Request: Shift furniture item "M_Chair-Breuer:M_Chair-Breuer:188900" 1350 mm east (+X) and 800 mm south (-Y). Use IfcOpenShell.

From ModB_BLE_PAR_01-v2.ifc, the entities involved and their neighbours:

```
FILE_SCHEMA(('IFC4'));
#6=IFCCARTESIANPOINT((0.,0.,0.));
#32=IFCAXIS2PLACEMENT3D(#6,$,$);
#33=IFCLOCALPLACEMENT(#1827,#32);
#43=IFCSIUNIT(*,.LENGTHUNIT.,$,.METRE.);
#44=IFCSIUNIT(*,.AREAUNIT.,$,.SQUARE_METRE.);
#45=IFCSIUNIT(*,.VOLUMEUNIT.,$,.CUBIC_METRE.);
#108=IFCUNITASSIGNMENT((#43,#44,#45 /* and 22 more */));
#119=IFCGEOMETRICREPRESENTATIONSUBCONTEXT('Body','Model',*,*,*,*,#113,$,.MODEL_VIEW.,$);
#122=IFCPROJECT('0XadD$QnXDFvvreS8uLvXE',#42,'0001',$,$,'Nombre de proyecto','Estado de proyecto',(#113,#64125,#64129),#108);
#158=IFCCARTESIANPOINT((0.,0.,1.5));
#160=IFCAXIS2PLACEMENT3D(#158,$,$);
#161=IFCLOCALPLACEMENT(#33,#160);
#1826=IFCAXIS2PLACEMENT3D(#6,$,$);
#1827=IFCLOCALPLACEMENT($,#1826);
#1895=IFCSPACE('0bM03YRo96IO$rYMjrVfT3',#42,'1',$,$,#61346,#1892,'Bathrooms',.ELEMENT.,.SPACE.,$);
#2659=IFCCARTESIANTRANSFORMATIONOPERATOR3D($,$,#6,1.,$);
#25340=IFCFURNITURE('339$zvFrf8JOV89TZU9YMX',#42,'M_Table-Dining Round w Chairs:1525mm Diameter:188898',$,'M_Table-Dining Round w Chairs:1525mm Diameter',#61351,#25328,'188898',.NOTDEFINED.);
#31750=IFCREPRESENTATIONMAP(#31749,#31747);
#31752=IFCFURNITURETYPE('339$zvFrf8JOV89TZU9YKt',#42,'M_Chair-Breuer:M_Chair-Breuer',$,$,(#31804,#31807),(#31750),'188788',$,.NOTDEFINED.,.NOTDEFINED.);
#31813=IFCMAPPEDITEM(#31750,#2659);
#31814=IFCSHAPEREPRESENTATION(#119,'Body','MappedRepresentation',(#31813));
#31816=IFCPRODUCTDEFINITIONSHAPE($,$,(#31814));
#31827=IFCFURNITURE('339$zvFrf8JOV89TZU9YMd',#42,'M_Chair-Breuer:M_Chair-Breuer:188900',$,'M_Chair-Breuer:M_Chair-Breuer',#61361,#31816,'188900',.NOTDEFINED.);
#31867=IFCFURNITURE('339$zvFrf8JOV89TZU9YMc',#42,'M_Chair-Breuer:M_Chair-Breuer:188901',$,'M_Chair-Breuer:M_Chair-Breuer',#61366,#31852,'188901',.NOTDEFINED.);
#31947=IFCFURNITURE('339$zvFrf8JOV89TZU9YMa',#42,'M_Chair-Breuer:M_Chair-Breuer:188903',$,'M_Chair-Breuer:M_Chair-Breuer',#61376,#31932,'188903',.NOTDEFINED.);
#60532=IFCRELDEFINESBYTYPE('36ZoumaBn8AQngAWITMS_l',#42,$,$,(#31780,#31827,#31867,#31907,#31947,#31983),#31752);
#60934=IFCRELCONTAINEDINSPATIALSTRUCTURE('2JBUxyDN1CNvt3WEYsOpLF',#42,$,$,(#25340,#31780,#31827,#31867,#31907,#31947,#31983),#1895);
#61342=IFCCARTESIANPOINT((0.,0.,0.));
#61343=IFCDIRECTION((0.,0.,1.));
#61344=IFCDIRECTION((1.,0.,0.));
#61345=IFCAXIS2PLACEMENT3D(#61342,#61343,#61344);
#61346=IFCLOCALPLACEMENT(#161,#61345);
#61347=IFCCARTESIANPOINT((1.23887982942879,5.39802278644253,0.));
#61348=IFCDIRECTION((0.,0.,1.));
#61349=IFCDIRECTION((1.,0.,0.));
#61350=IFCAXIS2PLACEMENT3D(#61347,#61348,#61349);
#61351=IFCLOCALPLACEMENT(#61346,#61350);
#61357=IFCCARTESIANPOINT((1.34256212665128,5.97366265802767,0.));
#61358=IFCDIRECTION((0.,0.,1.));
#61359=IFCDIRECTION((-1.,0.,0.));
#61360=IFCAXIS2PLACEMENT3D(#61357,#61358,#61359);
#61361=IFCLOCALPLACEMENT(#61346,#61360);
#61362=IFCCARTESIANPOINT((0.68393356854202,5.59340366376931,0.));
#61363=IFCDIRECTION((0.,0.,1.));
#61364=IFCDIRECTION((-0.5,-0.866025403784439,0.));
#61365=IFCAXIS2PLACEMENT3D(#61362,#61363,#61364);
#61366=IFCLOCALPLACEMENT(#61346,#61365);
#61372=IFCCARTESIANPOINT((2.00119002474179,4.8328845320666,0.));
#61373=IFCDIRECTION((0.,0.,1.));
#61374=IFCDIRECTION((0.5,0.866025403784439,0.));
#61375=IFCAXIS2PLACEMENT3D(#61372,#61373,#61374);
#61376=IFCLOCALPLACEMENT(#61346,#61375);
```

```python
import ifcopenshell
import ifcopenshell.api.geometry
import ifcopenshell.util.placement
import ifcopenshell.util.unit

model = ifcopenshell.open("ModB_BLE_PAR_01-v2.ifc")
unit_scale = ifcopenshell.util.unit.calculate_unit_scale(model)

item = model.by_guid("339$zvFrf8JOV89TZU9YMd")
matrix = ifcopenshell.util.placement.get_local_placement(item.ObjectPlacement)
matrix[0, 3] += 1.35 / unit_scale
matrix[1, 3] -= 0.8 / unit_scale
ifcopenshell.api.geometry.edit_object_placement(model, product=item, matrix=matrix, is_si=False)

print(ifcopenshell.util.placement.get_local_placement(item.ObjectPlacement).round(3) + 0.0)

model.write("ModB_BLE_PAR_01-v2_edited.ifc")
```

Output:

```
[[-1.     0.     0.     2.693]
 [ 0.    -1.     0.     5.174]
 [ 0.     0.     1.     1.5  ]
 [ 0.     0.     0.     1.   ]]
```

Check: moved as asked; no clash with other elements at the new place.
